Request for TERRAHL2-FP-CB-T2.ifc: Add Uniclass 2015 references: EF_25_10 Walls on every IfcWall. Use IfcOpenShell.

First a look at what the model holds.

```python
import ifcopenshell

model = ifcopenshell.open("TERRAHL2-FP-CB-T2.ifc")
print(model.schema)
print("classifications:", [c.Name for c in model.by_type("IfcClassification")])
for ifc_class in ("IfcDoor", "IfcRoof", "IfcStair", "IfcWall", "IfcWindow"):
    print(ifc_class, len(model.by_type(ifc_class)))
```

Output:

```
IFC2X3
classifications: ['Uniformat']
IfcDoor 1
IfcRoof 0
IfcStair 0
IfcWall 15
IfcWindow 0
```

```python
import ifcopenshell
import ifcopenshell.api.classification

model = ifcopenshell.open("TERRAHL2-FP-CB-T2.ifc")

# IFC2X3 requires Source and Edition and has no link from the project to the system.
system = model.create_entity("IfcClassification", Source="NBS", Edition="2015", Name="Uniclass 2015")

codes = {
    "IfcWall": ("EF_25_10", "Walls"),
}
for ifc_class, (code, name) in codes.items():
    products = model.by_type(ifc_class)
    ifcopenshell.api.classification.add_reference(
        model, products=products, classification=system, identification=code, name=name
    )
    print(code, len(products))

model.write("TERRAHL2-FP-CB-T2_edited.ifc")
```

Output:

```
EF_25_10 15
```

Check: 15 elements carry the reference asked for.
